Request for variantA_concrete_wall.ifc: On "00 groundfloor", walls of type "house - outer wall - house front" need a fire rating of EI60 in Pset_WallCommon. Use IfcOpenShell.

First a look at what the model holds.

```python
import ifcopenshell
import ifcopenshell.util.element

model = ifcopenshell.open("variantA_concrete_wall.ifc")
print(model.schema)
storey = next(s for s in model.by_type("IfcBuildingStorey") if s.Name == "00 groundfloor")
walls = [e for e in ifcopenshell.util.element.get_decomposition(storey) if e.is_a("IfcWall")]
seen = {}
for e in walls:
    element_type = ifcopenshell.util.element.get_type(e)
    key = (element_type.Name if element_type != e and element_type else None, ifcopenshell.util.element.get_pset(e, "Pset_WallCommon", "FireRating"))
    seen[key] = seen.get(key, 0) + 1
for (name, value), count in sorted(seen.items(), key=str):
    print(count, "x", name, "|", value)
```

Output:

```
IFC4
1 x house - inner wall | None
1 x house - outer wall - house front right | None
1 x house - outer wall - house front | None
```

```python
import ifcopenshell
import ifcopenshell.api.pset
import ifcopenshell.util.element

model = ifcopenshell.open("variantA_concrete_wall.ifc")

storey = next(s for s in model.by_type("IfcBuildingStorey") if s.Name == "00 groundfloor")
walls = [e for e in ifcopenshell.util.element.get_decomposition(storey) if e.is_a("IfcWall")]

count = 0
for e in walls:
    element_type = ifcopenshell.util.element.get_type(e)
    if element_type in (None, e) or element_type.Name != "house - outer wall - house front":
        continue
    # add_pset returns the element's existing set when there is one.
    pset = ifcopenshell.api.pset.add_pset(model, product=e, name="Pset_WallCommon")
    ifcopenshell.api.pset.edit_pset(model, pset=pset, properties={"FireRating": "EI60"})
    count += 1

print(count, "walls updated")

model.write("variantA_concrete_wall_v2.ifc")
```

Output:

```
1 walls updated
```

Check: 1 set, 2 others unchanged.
